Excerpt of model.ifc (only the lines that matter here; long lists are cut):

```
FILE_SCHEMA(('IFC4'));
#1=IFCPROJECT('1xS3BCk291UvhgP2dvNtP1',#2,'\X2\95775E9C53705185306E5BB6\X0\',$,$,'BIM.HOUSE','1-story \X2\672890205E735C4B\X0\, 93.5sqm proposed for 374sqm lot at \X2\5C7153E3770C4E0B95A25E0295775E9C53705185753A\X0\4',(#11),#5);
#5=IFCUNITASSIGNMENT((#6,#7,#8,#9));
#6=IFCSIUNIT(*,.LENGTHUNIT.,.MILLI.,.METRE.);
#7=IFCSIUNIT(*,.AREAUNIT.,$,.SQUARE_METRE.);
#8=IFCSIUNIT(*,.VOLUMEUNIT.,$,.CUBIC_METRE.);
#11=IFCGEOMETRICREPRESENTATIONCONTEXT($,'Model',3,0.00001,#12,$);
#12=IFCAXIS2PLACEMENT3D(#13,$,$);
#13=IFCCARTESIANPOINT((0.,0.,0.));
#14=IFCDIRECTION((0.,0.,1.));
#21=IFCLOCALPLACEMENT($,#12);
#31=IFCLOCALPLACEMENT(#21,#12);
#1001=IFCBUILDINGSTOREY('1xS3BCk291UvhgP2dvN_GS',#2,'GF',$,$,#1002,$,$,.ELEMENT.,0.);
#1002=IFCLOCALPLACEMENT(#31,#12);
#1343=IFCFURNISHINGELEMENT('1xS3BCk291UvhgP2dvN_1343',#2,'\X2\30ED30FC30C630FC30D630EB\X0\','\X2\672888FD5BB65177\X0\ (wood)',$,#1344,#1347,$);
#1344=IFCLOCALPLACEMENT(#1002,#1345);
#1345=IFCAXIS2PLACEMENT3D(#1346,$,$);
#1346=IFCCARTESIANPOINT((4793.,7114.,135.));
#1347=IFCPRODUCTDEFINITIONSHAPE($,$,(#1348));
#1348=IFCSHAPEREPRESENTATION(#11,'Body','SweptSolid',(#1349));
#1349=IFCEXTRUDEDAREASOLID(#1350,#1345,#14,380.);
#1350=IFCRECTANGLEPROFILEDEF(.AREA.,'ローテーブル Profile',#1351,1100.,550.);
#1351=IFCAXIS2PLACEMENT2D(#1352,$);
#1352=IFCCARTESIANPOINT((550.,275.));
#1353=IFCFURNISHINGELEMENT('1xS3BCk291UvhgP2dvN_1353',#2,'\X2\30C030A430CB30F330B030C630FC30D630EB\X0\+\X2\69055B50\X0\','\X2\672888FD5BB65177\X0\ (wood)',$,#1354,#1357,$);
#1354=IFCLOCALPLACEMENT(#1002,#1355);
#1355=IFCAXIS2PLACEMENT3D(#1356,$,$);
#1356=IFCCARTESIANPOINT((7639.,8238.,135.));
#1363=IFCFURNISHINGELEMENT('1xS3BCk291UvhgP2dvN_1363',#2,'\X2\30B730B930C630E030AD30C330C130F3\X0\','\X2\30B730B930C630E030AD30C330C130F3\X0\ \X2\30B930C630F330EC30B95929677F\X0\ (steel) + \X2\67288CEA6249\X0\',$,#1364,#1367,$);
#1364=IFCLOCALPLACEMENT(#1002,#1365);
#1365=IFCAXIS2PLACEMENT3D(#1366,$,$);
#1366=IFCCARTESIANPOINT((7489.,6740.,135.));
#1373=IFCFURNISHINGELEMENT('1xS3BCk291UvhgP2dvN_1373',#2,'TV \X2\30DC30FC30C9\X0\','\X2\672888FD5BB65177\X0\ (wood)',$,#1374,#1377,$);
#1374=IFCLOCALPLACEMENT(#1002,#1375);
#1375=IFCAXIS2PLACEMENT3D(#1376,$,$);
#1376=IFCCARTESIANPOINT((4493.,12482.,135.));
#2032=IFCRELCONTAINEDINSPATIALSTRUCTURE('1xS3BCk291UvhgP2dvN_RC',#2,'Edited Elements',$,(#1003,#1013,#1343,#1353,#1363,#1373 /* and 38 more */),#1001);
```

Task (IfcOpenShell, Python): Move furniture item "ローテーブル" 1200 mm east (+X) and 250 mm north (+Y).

```python
import ifcopenshell
import ifcopenshell.api.geometry
import ifcopenshell.util.placement

model = ifcopenshell.open("model.ifc")

item = model.by_guid("1xS3BCk291UvhgP2dvN_1343")
matrix = ifcopenshell.util.placement.get_local_placement(item.ObjectPlacement)
matrix[0, 3] += 1200.0
matrix[1, 3] += 250.0
ifcopenshell.api.geometry.edit_object_placement(model, product=item, matrix=matrix, is_si=False)

print(ifcopenshell.util.placement.get_local_placement(item.ObjectPlacement).round(3) + 0.0)

model.write("model_edited.ifc")
```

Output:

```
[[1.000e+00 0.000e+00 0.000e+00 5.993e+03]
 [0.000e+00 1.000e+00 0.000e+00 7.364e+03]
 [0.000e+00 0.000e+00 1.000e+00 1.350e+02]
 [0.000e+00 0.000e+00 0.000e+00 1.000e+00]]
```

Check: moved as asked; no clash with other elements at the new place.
